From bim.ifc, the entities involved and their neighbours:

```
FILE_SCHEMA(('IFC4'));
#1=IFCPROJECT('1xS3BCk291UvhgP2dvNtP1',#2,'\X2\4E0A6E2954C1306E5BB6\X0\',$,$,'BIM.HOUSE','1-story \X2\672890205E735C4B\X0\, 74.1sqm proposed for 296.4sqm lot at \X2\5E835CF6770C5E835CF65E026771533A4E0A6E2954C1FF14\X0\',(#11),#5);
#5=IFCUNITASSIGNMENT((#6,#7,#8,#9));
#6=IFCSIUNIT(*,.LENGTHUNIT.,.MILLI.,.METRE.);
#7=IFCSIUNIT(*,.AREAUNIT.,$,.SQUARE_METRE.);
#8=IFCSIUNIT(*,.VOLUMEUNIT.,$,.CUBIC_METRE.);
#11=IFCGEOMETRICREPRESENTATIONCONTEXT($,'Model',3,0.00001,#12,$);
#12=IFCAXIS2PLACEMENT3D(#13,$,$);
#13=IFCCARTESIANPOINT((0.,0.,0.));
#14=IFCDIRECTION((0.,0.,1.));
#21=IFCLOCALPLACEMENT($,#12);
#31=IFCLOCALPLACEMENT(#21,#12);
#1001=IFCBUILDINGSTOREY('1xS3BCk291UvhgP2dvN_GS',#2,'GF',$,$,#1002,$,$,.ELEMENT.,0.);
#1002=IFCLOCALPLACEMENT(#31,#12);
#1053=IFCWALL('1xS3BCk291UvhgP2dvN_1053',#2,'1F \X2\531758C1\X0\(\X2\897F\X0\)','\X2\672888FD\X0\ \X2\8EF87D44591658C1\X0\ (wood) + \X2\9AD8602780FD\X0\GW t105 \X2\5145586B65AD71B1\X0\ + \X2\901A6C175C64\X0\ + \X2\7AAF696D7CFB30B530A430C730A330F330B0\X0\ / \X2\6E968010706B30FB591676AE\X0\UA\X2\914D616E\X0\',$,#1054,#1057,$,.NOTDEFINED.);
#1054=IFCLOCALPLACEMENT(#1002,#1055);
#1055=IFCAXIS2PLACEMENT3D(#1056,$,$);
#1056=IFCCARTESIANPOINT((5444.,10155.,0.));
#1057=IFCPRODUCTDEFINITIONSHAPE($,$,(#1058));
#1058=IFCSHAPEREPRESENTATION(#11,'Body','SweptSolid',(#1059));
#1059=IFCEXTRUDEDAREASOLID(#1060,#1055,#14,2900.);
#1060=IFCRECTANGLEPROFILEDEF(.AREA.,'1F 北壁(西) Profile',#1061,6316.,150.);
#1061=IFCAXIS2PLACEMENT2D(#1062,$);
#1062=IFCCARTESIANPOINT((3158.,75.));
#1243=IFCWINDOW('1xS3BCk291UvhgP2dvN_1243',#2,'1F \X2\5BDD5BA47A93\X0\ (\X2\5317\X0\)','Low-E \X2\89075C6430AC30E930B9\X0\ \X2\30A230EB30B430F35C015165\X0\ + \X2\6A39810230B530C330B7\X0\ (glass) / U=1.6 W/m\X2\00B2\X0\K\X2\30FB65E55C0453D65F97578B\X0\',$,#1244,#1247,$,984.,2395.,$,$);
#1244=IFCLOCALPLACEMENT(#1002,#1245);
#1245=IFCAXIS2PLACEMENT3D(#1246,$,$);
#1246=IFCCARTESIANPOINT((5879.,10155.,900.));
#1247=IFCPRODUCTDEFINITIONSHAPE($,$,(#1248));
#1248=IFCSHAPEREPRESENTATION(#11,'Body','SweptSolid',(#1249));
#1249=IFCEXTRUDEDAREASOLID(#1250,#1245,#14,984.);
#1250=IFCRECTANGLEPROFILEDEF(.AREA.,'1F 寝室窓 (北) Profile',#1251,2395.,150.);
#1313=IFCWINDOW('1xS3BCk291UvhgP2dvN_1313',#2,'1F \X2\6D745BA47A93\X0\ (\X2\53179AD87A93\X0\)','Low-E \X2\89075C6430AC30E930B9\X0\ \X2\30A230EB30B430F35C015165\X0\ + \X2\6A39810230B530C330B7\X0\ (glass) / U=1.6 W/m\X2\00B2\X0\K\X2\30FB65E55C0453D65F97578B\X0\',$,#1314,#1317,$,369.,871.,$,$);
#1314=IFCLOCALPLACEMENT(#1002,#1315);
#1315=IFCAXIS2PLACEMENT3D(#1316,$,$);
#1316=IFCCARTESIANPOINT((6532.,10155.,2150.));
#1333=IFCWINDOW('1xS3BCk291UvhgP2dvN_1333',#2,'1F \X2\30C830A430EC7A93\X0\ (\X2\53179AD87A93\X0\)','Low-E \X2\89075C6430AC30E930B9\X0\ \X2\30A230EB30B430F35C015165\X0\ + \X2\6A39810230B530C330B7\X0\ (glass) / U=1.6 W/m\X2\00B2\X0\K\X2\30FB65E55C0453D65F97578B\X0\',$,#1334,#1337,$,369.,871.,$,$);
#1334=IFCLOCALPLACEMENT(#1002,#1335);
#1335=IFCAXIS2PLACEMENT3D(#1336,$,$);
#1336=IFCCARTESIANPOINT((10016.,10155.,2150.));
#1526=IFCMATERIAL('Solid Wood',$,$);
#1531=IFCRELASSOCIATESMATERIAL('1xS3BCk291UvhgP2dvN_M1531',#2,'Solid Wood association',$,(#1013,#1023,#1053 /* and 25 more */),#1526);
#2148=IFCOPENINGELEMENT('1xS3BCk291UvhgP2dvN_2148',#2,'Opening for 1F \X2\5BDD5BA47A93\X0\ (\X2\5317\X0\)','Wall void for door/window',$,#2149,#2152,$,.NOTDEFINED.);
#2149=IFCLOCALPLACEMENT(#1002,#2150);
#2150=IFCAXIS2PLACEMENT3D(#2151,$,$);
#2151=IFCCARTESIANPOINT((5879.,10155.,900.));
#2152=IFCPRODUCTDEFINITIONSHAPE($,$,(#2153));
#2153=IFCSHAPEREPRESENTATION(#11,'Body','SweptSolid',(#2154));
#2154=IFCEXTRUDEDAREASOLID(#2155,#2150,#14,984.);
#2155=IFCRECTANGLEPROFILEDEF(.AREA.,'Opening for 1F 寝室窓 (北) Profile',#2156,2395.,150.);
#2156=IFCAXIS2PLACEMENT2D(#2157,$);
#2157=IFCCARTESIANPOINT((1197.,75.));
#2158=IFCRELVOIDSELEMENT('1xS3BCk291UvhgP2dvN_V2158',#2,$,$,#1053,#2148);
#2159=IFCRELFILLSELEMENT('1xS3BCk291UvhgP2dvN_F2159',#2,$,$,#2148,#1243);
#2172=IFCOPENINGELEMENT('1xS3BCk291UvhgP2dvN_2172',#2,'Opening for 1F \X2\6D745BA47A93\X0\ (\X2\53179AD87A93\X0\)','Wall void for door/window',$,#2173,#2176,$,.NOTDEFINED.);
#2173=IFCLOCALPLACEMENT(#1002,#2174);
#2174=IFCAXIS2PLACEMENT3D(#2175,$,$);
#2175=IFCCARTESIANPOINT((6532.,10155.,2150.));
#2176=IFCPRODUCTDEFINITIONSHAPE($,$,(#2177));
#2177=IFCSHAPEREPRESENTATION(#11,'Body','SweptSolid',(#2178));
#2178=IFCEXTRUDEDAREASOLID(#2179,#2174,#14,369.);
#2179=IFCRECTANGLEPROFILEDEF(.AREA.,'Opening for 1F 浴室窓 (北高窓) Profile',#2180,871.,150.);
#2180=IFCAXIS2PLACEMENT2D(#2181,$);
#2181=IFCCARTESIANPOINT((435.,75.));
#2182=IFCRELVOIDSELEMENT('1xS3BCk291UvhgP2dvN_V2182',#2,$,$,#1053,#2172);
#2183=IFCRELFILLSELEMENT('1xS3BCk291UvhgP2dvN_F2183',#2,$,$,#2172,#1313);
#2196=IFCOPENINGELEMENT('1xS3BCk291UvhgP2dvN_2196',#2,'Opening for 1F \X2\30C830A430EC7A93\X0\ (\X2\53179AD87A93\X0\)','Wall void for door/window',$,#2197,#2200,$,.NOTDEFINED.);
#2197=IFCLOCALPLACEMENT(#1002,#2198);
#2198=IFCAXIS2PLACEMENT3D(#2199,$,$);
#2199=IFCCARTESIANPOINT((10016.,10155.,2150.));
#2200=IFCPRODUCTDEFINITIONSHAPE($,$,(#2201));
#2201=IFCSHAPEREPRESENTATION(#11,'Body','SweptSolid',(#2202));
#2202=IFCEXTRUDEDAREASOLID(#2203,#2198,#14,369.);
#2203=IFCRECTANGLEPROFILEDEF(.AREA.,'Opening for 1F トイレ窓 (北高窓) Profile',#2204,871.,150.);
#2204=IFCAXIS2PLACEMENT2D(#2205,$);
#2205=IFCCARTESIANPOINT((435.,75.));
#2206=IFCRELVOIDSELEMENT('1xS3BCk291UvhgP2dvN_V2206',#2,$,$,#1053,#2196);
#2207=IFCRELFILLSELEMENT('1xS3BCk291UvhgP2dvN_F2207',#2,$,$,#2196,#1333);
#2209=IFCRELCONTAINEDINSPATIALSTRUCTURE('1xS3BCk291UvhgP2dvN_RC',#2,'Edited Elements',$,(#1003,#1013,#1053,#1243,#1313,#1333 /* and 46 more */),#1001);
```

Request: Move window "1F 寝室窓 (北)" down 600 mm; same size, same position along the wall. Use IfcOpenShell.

```python
import numpy as np
import ifcopenshell
import ifcopenshell.api.geometry
import ifcopenshell.util.placement
import ifcopenshell.util.unit

model = ifcopenshell.open("bim.ifc")
unit_scale = ifcopenshell.util.unit.calculate_unit_scale(model)

window = model.by_guid("1xS3BCk291UvhgP2dvN_1243")
opening = window.FillsVoids[0].RelatingOpeningElement
dz = -0.6 / unit_scale

shift = np.array([0.0, 0.0, dz])
# The window is not placed relative to its opening, so move both.
for product in (opening, window):
    matrix = ifcopenshell.util.placement.get_local_placement(product.ObjectPlacement)
    matrix[:3, 3] += shift
    ifcopenshell.api.geometry.edit_object_placement(model, product=product, matrix=matrix, is_si=False)

print(f"moved by {dz * unit_scale:+.3f} m")

model.write("bim-out.ifc")
```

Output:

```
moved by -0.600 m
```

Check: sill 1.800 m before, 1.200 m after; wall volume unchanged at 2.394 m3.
